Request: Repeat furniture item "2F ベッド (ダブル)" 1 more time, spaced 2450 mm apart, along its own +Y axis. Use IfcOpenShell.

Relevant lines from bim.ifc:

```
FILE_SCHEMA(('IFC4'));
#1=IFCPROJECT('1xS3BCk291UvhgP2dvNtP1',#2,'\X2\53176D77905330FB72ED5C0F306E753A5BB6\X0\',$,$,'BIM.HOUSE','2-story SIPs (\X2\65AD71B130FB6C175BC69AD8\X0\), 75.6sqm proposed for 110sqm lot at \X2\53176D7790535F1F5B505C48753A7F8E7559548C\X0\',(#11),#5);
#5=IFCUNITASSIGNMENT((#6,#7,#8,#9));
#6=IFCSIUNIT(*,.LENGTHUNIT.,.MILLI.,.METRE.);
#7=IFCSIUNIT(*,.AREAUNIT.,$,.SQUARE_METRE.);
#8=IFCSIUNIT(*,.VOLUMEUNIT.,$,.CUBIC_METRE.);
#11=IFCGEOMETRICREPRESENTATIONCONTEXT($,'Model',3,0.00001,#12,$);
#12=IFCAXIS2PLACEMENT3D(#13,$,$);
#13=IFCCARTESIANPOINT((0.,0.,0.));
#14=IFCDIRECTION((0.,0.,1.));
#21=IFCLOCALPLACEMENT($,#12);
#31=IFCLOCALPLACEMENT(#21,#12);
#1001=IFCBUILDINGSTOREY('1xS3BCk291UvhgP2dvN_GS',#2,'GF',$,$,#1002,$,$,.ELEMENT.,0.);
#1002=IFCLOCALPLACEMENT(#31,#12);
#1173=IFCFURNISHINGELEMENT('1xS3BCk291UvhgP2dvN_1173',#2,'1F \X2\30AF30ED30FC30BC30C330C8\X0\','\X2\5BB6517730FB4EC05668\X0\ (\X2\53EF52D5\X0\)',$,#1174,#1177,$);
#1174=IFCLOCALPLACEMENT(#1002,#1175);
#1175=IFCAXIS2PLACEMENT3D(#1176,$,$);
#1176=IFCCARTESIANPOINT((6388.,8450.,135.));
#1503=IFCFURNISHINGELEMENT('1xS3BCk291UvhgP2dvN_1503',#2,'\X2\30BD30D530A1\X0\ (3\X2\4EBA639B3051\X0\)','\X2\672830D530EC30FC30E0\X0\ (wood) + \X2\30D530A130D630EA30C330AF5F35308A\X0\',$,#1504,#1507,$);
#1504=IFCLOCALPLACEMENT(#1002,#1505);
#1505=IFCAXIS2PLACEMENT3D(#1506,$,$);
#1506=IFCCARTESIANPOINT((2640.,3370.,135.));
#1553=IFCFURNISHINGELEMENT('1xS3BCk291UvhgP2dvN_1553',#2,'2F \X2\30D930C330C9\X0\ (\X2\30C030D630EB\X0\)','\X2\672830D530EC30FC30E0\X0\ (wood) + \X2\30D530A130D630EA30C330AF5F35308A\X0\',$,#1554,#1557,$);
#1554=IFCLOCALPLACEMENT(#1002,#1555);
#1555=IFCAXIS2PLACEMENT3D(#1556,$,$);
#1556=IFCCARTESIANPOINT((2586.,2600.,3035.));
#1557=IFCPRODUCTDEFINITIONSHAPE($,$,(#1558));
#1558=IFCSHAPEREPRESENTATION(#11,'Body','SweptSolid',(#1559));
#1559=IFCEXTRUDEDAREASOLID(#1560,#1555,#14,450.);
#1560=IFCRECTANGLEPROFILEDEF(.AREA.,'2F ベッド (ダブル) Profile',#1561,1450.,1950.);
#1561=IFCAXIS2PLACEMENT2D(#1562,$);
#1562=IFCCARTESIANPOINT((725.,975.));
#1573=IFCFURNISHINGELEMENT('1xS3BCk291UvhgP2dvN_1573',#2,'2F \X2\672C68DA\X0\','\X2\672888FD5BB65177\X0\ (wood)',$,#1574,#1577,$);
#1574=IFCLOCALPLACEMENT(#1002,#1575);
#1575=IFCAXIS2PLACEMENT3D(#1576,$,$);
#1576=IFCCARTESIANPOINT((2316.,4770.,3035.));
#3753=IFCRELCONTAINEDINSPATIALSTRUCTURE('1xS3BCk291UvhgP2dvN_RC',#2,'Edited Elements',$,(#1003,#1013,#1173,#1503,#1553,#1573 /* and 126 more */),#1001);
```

```python
import ifcopenshell
import ifcopenshell.api.geometry
import ifcopenshell.api.root
import ifcopenshell.util.element
import ifcopenshell.util.placement

model = ifcopenshell.open("bim.ifc")


def reuse_history(source, copy):
    """copy_class also copies each property set's owner history, people and application; keep the originals."""
    for rel in copy.IsDefinedBy:
        if rel.is_a("IfcRelDefinesByProperties") and (history := rel.RelatingPropertyDefinition.OwnerHistory):
            rel.RelatingPropertyDefinition.OwnerHistory = source.OwnerHistory
            ifcopenshell.util.element.remove_deep2(model, history)


source = model.by_id(1553)
base = ifcopenshell.util.placement.get_local_placement(source.ObjectPlacement)
step = base[:3, 1] * 2450.0

for i in range(1, 2):
    copy = ifcopenshell.api.root.copy_class(model, product=source)
    copy.Representation = ifcopenshell.util.element.copy_deep(
        model, source.Representation, exclude=["IfcGeometricRepresentationContext", "IfcRepresentationMap"]
    )
    reuse_history(source, copy)
    matrix = base.copy()
    matrix[:3, 3] += i * step
    print("added at", matrix[:3, 3].round(3) + 0.0)
    ifcopenshell.api.geometry.edit_object_placement(model, product=copy, matrix=matrix, is_si=False)

model.write("bim_edited.ifc")
```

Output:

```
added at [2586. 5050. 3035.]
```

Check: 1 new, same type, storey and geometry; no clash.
